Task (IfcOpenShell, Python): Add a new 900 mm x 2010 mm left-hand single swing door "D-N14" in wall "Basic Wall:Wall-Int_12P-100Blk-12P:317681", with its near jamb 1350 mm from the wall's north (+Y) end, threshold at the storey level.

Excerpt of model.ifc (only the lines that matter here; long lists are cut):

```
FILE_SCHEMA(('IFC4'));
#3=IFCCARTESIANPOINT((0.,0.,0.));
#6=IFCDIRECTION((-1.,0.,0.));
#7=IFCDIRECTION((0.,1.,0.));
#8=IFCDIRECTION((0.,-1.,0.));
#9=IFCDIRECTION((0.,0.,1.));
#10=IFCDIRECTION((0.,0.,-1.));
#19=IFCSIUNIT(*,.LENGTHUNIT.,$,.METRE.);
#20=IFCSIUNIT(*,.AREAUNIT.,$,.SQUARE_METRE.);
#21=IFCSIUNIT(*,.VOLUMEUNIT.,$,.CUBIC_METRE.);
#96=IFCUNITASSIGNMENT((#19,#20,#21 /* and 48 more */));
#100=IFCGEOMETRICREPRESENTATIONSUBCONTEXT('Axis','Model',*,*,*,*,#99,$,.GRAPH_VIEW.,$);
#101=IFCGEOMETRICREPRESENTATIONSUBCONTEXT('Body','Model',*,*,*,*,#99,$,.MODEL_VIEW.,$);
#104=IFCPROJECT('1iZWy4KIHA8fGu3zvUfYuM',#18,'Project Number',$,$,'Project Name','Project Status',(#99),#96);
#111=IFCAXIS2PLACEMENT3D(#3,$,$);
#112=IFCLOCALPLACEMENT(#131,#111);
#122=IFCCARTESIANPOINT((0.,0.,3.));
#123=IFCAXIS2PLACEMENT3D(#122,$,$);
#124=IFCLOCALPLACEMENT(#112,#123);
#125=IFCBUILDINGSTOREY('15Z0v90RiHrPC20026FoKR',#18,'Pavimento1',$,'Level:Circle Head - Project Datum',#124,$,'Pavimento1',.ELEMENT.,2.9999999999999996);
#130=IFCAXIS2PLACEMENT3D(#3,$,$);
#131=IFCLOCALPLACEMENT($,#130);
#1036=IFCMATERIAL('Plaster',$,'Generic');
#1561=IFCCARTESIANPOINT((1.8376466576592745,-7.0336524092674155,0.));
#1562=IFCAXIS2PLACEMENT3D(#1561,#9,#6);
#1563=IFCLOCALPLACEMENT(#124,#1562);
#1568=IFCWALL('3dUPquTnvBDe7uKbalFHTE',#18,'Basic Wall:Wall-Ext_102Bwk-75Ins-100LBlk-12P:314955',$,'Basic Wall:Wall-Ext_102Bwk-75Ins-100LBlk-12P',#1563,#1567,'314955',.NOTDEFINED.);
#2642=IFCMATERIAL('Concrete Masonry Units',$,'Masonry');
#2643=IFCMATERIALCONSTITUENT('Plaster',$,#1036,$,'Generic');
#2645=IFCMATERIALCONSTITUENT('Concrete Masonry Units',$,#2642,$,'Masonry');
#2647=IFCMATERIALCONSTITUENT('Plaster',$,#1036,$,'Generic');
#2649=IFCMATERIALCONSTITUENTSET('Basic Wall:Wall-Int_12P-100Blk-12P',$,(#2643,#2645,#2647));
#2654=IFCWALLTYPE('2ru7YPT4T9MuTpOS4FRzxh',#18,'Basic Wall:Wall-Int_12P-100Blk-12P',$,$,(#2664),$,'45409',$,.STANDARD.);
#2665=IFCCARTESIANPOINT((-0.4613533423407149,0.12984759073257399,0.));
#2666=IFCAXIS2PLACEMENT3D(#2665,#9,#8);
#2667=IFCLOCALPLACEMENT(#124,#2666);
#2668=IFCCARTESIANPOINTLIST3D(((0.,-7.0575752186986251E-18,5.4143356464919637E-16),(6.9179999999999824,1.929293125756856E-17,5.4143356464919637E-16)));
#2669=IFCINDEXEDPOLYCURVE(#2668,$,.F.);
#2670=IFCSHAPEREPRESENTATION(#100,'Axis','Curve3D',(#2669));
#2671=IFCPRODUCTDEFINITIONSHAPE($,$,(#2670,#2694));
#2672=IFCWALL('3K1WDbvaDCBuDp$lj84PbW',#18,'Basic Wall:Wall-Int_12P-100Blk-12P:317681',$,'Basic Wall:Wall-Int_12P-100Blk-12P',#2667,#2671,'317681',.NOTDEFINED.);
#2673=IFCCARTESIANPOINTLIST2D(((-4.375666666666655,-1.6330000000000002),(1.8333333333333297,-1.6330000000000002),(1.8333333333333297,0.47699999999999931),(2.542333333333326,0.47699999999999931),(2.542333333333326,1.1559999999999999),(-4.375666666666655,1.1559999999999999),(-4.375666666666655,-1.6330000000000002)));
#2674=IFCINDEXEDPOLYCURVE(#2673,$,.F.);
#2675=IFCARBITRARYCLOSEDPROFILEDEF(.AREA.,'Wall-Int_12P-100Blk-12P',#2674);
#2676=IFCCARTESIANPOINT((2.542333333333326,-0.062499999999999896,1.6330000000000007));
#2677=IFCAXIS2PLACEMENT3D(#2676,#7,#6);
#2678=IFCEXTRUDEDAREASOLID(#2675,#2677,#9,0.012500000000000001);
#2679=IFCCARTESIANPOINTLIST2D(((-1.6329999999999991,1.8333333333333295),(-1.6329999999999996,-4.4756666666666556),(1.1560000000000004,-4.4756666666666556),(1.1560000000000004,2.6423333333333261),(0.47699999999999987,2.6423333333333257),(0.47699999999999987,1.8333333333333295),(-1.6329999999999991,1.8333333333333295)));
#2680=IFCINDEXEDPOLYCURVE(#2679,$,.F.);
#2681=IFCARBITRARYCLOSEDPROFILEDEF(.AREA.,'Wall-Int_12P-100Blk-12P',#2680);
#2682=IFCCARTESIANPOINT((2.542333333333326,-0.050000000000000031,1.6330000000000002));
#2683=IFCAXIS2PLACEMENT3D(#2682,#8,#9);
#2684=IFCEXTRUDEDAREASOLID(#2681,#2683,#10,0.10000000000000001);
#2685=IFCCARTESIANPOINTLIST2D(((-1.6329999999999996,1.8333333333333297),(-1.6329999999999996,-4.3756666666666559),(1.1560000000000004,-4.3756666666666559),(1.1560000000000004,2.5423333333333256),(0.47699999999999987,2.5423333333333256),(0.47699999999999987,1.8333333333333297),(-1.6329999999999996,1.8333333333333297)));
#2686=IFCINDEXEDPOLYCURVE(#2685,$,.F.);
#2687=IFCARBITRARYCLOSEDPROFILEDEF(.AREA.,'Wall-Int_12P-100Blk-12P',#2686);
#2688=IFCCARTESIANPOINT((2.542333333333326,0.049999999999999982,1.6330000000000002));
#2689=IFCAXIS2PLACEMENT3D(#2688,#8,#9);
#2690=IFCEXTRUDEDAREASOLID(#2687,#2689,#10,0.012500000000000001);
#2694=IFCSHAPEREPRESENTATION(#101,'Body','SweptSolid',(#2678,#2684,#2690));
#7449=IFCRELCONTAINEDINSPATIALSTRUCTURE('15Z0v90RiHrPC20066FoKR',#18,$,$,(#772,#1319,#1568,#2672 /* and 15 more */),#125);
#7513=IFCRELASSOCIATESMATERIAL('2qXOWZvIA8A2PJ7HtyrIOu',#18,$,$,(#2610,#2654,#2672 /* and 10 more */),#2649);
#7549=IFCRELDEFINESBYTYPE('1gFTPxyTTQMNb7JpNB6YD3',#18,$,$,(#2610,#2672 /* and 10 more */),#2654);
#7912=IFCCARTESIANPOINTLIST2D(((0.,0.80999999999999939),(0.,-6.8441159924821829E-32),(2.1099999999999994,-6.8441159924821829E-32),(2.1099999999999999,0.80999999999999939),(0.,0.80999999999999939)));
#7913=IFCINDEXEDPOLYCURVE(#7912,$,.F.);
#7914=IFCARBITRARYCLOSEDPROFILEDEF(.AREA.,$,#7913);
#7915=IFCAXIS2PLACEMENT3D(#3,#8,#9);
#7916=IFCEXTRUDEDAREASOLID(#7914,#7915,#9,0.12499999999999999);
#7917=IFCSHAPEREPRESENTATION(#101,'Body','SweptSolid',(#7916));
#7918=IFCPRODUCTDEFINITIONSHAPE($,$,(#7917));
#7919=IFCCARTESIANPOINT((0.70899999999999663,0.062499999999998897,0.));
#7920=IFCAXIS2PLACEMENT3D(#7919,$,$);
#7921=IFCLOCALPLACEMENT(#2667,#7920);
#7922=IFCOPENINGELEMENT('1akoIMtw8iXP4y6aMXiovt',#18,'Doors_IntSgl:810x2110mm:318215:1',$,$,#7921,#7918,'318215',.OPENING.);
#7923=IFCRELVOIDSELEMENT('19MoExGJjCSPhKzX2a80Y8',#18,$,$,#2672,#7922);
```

```python
import numpy as np
import ifcopenshell
import ifcopenshell.api.feature
import ifcopenshell.api.geometry
import ifcopenshell.api.root
import ifcopenshell.api.spatial
import ifcopenshell.geom
import ifcopenshell.util.element
import ifcopenshell.util.placement
import ifcopenshell.util.representation
import ifcopenshell.util.shape
import ifcopenshell.util.unit

model = ifcopenshell.open("model.ifc")
unit_scale = ifcopenshell.util.unit.calculate_unit_scale(model)
settings = ifcopenshell.geom.settings()


def volume(element):
    """Net volume in cubic metres, openings subtracted."""
    shape = ifcopenshell.geom.create_shape(settings, element)
    return ifcopenshell.util.shape.get_volume(shape.geometry)


wall = model.by_id(2672)
storey = ifcopenshell.util.element.get_container(wall, ifc_class="IfcBuildingStorey")
context = ifcopenshell.util.representation.get_context(model, "Model", "Body", "MODEL_VIEW")
before = volume(wall)

width, height, from_end, sill = 0.9, 2.01, 1.35, 0.0  # metres

# The wall runs along its own X axis, and the end named is its -X end.
wall_shape = ifcopenshell.geom.create_shape(settings, wall)
x, y, z = ifcopenshell.util.shape.get_vertices(wall_shape.geometry).T
start = x.min() + from_end
face, thickness = float(y.min()), float(y.max() - y.min())
wall_matrix = ifcopenshell.util.placement.get_local_placement(wall.ObjectPlacement)
level = ifcopenshell.util.placement.get_local_placement(storey.ObjectPlacement)[2, 3]


def in_wall(x, y):
    """Placement at x, y metres in the wall's axes, at sill height."""
    matrix = wall_matrix.copy()
    matrix[:, 3] = wall_matrix @ np.array([x / unit_scale, y / unit_scale, 0.0, 1.0])
    matrix[2, 3] = level + sill / unit_scale
    return matrix


# Opening: a box that overshoots both wall faces by 50 mm.
opening = ifcopenshell.api.root.create_entity(model, ifc_class="IfcOpeningElement", predefined_type="OPENING")
box = ifcopenshell.api.geometry.add_wall_representation(
    model, context=context, length=width, height=height, thickness=thickness + 0.1
)
ifcopenshell.api.geometry.assign_representation(model, product=opening, representation=box)
ifcopenshell.api.geometry.edit_object_placement(model, product=opening, matrix=in_wall(start, face - 0.05), is_si=False)
ifcopenshell.api.feature.add_feature(model, feature=opening, element=wall)

door = ifcopenshell.api.root.create_entity(model, ifc_class="IfcDoor", name="D-N14", predefined_type="DOOR")
door.OverallWidth, door.OverallHeight = width / unit_scale, height / unit_scale
door.OperationType = "SINGLE_SWING_LEFT"
body = ifcopenshell.api.geometry.add_door_representation(
    model,
    context=context,
    overall_width=door.OverallWidth,
    overall_height=door.OverallHeight,
    operation_type="SINGLE_SWING_LEFT",
    lining_properties={"LiningDepth": thickness / unit_scale, "ThresholdDepth": thickness / unit_scale},
)
ifcopenshell.api.geometry.assign_representation(model, product=door, representation=body)
ifcopenshell.api.spatial.assign_container(model, products=[door], relating_structure=storey)
ifcopenshell.api.feature.add_filling(model, opening=opening, element=door)

# The lining spans the wall, so the door starts at the wall face.
ifcopenshell.api.geometry.edit_object_placement(model, product=door, matrix=in_wall(start, face), is_si=False)

after = volume(wall)

print(f"wall volume {before:.3f} -> {after:.3f} m3")

model.write("model_updated.ifc")
```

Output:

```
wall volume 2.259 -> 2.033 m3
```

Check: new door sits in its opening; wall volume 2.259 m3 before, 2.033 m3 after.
